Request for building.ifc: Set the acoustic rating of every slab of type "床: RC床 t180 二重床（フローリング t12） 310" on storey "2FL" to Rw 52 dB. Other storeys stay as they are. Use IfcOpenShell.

First a look at what the model holds.

```python
import ifcopenshell
import ifcopenshell.util.element

model = ifcopenshell.open("building.ifc")
print(model.schema)
storey = next(s for s in model.by_type("IfcBuildingStorey") if s.Name == "2FL")
slabs = [e for e in ifcopenshell.util.element.get_decomposition(storey) if e.is_a("IfcSlab")]
seen = {}
for e in slabs:
    element_type = ifcopenshell.util.element.get_type(e)
    key = (element_type.Name if element_type != e and element_type else None, ifcopenshell.util.element.get_pset(e, "Pset_SlabCommon", "AcousticRating"))
    seen[key] = seen.get(key, 0) + 1
for (name, value), count in sorted(seen.items(), key=str):
    print(count, "x", name, "|", value)
```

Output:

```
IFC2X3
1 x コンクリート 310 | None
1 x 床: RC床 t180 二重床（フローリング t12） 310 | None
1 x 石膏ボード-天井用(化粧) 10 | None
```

```python
import ifcopenshell
import ifcopenshell.api.pset
import ifcopenshell.util.element

model = ifcopenshell.open("building.ifc")

storey = next(s for s in model.by_type("IfcBuildingStorey") if s.Name == "2FL")
slabs = [e for e in ifcopenshell.util.element.get_decomposition(storey) if e.is_a("IfcSlab")]

count = 0
for e in slabs:
    element_type = ifcopenshell.util.element.get_type(e)
    if element_type in (None, e) or element_type.Name != "床: RC床 t180 二重床（フローリング t12） 310":
        continue
    # add_pset returns the element's existing set when there is one.
    pset = ifcopenshell.api.pset.add_pset(model, product=e, name="Pset_SlabCommon")
    ifcopenshell.api.pset.edit_pset(model, pset=pset, properties={"AcousticRating": "Rw 52 dB"})
    count += 1

print(count, "slabs updated")

model.write("building-out.ifc")
```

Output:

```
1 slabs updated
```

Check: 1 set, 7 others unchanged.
